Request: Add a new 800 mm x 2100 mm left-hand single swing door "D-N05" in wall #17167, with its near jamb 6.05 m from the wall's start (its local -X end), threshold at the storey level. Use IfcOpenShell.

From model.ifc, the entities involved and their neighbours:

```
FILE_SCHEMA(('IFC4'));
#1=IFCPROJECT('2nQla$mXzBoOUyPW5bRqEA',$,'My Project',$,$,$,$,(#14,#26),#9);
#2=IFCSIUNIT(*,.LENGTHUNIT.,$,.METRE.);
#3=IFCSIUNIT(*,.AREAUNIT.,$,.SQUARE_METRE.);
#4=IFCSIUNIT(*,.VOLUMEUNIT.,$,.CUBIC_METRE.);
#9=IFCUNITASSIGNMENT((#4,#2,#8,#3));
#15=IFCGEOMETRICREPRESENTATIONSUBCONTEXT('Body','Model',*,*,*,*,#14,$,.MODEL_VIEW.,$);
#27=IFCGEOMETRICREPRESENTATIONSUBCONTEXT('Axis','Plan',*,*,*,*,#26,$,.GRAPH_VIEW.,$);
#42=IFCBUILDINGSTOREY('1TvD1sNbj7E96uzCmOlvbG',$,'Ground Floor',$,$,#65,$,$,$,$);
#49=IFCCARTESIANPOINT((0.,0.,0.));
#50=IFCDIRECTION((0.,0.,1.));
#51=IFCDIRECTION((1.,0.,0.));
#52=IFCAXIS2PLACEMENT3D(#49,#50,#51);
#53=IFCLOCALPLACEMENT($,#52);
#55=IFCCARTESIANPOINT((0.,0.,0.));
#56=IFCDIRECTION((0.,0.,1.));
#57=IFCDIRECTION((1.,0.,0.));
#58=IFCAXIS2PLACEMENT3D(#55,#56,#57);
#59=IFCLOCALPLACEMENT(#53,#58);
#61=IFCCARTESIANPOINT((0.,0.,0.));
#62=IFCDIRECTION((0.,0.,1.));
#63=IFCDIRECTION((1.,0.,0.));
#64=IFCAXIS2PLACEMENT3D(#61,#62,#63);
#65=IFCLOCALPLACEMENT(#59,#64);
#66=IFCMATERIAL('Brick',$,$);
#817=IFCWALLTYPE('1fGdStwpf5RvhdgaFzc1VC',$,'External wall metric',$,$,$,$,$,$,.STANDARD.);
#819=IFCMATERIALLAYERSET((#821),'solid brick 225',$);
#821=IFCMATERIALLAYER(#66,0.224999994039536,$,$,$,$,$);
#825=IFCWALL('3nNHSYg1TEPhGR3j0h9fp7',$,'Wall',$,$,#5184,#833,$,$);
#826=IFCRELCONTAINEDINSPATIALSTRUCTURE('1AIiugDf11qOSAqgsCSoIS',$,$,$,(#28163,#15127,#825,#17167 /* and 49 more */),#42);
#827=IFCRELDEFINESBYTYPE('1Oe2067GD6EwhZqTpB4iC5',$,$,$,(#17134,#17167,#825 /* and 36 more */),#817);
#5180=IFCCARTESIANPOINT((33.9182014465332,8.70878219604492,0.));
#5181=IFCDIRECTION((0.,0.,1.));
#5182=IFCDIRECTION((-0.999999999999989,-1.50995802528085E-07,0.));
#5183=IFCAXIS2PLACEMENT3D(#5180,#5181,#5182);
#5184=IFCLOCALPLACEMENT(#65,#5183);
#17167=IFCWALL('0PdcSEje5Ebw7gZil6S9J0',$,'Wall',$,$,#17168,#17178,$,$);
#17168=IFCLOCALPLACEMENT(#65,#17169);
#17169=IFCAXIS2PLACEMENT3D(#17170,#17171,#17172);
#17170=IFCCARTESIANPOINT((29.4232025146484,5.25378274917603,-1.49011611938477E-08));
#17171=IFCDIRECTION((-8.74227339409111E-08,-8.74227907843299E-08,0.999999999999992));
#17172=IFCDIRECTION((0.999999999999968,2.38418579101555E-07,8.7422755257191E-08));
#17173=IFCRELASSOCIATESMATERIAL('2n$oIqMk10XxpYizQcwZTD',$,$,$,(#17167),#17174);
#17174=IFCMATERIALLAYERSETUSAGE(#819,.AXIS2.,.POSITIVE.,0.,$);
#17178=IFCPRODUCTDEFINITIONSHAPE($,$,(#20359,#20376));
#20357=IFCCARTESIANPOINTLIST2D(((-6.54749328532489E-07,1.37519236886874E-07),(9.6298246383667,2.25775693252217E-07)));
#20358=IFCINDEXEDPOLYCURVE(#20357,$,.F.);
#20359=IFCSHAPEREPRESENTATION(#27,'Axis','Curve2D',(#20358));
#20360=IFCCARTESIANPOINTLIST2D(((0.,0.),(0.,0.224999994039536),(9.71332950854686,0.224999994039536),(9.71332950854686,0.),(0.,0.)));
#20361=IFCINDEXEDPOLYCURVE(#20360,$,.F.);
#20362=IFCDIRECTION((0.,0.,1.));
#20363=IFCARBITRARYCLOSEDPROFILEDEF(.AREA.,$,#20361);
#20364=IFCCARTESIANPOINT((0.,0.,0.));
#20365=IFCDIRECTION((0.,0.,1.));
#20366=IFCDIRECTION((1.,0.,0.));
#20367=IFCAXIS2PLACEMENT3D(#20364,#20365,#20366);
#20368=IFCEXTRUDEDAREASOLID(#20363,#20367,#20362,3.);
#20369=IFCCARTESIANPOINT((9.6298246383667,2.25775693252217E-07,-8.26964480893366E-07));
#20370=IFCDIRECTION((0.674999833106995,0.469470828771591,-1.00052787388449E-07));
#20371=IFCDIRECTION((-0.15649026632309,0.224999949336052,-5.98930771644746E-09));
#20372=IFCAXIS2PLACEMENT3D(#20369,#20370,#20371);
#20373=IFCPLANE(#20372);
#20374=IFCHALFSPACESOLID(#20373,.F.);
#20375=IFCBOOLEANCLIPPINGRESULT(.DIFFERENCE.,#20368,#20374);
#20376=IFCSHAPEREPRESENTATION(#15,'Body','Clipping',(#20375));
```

```python
import numpy as np
import ifcopenshell
import ifcopenshell.api.feature
import ifcopenshell.api.geometry
import ifcopenshell.api.root
import ifcopenshell.api.spatial
import ifcopenshell.geom
import ifcopenshell.util.element
import ifcopenshell.util.placement
import ifcopenshell.util.representation
import ifcopenshell.util.shape
import ifcopenshell.util.unit

model = ifcopenshell.open("model.ifc")
unit_scale = ifcopenshell.util.unit.calculate_unit_scale(model)
settings = ifcopenshell.geom.settings()


def volume(element):
    """Net volume in cubic metres, openings subtracted."""
    shape = ifcopenshell.geom.create_shape(settings, element)
    return ifcopenshell.util.shape.get_volume(shape.geometry)


wall = model.by_guid("0PdcSEje5Ebw7gZil6S9J0")
storey = ifcopenshell.util.element.get_container(wall, ifc_class="IfcBuildingStorey")
context = ifcopenshell.util.representation.get_context(model, "Model", "Body", "MODEL_VIEW")
before = volume(wall)

width, height, from_end, sill = 0.8, 2.1, 6.05, 0.0  # metres

# The wall runs along its own X axis, and the end named is its -X end.
wall_shape = ifcopenshell.geom.create_shape(settings, wall)
x, y, z = ifcopenshell.util.shape.get_vertices(wall_shape.geometry).T
start = x.min() + from_end
face, thickness = float(y.min()), float(y.max() - y.min())
wall_matrix = ifcopenshell.util.placement.get_local_placement(wall.ObjectPlacement)
level = ifcopenshell.util.placement.get_local_placement(storey.ObjectPlacement)[2, 3]


def in_wall(x, y):
    """Placement at x, y metres in the wall's axes, at sill height."""
    matrix = wall_matrix.copy()
    matrix[:, 3] = wall_matrix @ np.array([x / unit_scale, y / unit_scale, 0.0, 1.0])
    matrix[2, 3] = level + sill / unit_scale
    return matrix


# Opening: a box that overshoots both wall faces by 50 mm.
opening = ifcopenshell.api.root.create_entity(model, ifc_class="IfcOpeningElement", predefined_type="OPENING")
box = ifcopenshell.api.geometry.add_wall_representation(
    model, context=context, length=width, height=height, thickness=thickness + 0.1
)
ifcopenshell.api.geometry.assign_representation(model, product=opening, representation=box)
ifcopenshell.api.geometry.edit_object_placement(model, product=opening, matrix=in_wall(start, face - 0.05), is_si=False)
ifcopenshell.api.feature.add_feature(model, feature=opening, element=wall)

door = ifcopenshell.api.root.create_entity(model, ifc_class="IfcDoor", name="D-N05", predefined_type="DOOR")
door.OverallWidth, door.OverallHeight = width / unit_scale, height / unit_scale
door.OperationType = "SINGLE_SWING_LEFT"
body = ifcopenshell.api.geometry.add_door_representation(
    model,
    context=context,
    overall_width=door.OverallWidth,
    overall_height=door.OverallHeight,
    operation_type="SINGLE_SWING_LEFT",
    lining_properties={"LiningDepth": thickness / unit_scale, "ThresholdDepth": thickness / unit_scale},
)
ifcopenshell.api.geometry.assign_representation(model, product=door, representation=body)
ifcopenshell.api.spatial.assign_container(model, products=[door], relating_structure=storey)
ifcopenshell.api.feature.add_filling(model, opening=opening, element=door)

# The lining spans the wall, so the door starts at the wall face.
ifcopenshell.api.geometry.edit_object_placement(model, product=door, matrix=in_wall(start, face), is_si=False)

after = volume(wall)

print(f"wall volume {before:.3f} -> {after:.3f} m3")

model.write("model-out.ifc")
```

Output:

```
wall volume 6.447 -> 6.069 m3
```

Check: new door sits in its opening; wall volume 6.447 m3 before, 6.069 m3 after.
